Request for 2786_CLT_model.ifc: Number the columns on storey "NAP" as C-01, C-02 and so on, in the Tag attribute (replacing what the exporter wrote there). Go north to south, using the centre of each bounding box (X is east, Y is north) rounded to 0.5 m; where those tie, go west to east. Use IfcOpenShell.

First a look at what the model holds.

```python
import ifcopenshell
import ifcopenshell.util.element
import ifcopenshell.util.placement

model = ifcopenshell.open("2786_CLT_model.ifc")
print(model.schema)
storey = next(s for s in model.by_type("IfcBuildingStorey") if s.Name == "NAP")
columns = [e for e in ifcopenshell.util.element.get_decomposition(storey) if e.is_a("IfcColumn")]
for e in sorted(columns, key=lambda e: e.id()):
    origin = ifcopenshell.util.placement.get_local_placement(e.ObjectPlacement)[:3, 3]
    print(e.id(), e.Tag, e.Name, origin.round(2) + 0.0, sep=" | ")
```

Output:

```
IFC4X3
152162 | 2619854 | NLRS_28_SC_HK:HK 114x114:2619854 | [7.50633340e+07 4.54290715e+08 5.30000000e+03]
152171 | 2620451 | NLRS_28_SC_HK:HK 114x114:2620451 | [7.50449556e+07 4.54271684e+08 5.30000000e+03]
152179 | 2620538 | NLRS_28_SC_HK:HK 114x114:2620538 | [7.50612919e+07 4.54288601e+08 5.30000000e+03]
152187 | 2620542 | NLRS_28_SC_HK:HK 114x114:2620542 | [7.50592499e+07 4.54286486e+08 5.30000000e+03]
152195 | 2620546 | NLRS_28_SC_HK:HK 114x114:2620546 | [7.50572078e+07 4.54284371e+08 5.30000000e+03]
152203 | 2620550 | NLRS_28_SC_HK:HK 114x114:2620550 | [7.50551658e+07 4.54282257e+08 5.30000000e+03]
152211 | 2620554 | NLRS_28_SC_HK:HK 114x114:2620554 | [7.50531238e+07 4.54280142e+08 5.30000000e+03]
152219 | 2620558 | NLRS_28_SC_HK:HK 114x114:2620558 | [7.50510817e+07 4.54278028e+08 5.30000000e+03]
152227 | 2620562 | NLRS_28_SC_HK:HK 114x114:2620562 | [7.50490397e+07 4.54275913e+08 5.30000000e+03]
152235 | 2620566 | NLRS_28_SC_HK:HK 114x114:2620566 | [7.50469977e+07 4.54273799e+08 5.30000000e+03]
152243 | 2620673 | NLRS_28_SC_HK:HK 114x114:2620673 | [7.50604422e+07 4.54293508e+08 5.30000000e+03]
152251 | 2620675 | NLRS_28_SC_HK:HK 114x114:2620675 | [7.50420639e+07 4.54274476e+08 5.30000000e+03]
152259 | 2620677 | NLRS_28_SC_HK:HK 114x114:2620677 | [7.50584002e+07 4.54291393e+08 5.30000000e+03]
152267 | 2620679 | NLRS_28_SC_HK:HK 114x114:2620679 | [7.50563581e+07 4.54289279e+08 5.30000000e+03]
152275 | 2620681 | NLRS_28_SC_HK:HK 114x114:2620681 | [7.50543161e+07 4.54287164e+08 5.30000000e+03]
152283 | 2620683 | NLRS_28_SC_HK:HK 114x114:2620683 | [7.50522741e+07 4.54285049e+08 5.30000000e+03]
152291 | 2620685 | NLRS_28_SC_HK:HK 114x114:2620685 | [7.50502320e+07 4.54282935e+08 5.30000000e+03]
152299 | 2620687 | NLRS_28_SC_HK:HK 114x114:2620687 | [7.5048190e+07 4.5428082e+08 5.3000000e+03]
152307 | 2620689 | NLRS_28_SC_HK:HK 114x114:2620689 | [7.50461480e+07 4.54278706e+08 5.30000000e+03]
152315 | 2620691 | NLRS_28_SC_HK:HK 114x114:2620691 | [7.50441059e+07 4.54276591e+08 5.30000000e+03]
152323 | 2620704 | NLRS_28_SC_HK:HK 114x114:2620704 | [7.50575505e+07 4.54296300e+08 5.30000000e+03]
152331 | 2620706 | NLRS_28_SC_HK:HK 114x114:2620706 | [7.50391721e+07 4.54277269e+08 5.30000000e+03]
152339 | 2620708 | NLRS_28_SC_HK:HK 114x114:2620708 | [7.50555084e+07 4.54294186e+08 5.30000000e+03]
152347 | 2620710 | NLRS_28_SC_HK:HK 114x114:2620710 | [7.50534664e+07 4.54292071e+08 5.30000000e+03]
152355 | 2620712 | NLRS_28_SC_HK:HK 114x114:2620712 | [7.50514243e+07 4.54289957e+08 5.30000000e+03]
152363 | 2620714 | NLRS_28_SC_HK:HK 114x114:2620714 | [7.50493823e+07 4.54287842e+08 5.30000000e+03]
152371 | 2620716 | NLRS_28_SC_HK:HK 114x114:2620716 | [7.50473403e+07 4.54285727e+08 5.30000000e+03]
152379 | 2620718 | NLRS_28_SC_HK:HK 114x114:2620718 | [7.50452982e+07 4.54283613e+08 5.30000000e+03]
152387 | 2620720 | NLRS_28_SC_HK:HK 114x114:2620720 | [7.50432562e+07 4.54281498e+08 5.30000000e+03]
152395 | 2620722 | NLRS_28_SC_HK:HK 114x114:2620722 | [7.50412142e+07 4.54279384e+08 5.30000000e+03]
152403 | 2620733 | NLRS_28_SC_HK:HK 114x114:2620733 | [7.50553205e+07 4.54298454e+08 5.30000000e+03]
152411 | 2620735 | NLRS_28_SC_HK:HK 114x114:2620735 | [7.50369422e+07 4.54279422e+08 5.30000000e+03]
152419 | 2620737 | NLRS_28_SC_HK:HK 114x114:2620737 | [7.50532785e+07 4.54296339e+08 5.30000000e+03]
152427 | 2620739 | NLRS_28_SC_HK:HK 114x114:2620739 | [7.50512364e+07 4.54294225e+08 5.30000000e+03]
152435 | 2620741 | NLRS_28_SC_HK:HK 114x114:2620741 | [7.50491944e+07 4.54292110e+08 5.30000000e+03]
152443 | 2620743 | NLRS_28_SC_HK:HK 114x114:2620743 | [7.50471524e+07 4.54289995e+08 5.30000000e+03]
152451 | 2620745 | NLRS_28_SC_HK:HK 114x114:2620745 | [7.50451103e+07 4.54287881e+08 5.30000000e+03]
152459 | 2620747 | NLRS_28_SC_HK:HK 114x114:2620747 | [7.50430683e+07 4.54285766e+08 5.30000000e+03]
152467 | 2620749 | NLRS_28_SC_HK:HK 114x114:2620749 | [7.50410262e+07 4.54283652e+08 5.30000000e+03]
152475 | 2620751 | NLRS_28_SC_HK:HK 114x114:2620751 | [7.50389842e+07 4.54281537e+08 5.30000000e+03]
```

```python
import ifcopenshell
import ifcopenshell.geom
import ifcopenshell.util.element
import ifcopenshell.util.shape

model = ifcopenshell.open("2786_CLT_model.ifc")
settings = ifcopenshell.geom.settings()
settings.set("use-world-coords", True)


def centre(element):
    shape = ifcopenshell.geom.create_shape(settings, element)
    return ifcopenshell.util.shape.get_bbox_centroid(shape.geometry)


storey = next(s for s in model.by_type("IfcBuildingStorey") if s.Name == "NAP")
columns = [e for e in ifcopenshell.util.element.get_decomposition(storey) if e.is_a("IfcColumn")]

# Insertion points can sit at a corner or the storey origin, so sort by the geometry (in metres).
centres = {e: centre(e) for e in columns}
columns.sort(key=lambda e: (-round(centres[e][1] / 0.5), centres[e][0]))

for i, e in enumerate(columns, start=1):
    number = f"C-{i:02d}"
    e.Tag = number
    print(e.id(), number)

model.write("2786_CLT_model_edited.ifc")
```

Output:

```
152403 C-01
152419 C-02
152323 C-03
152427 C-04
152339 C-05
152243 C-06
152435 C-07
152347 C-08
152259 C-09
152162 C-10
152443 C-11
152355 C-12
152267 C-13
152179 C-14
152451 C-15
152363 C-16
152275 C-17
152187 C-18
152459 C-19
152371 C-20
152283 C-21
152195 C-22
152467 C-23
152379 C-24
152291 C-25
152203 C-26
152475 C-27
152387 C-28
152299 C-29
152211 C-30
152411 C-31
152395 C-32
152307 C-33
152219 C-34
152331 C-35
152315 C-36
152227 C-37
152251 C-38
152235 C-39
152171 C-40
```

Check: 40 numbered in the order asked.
